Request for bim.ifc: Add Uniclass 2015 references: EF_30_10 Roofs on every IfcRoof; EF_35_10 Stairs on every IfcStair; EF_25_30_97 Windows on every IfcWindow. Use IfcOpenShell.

First a look at what the model holds.

```python
import ifcopenshell

model = ifcopenshell.open("bim.ifc")
print(model.schema)
print("classifications:", [c.Name for c in model.by_type("IfcClassification")])
for ifc_class in ("IfcDoor", "IfcRoof", "IfcStair", "IfcWall", "IfcWindow"):
    print(ifc_class, len(model.by_type(ifc_class)))
```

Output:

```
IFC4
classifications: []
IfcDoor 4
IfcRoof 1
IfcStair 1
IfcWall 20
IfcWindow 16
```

```python
import ifcopenshell
import ifcopenshell.api.classification

model = ifcopenshell.open("bim.ifc")

system = ifcopenshell.api.classification.add_classification(model, classification="Uniclass 2015")

codes = {
    "IfcRoof": ("EF_30_10", "Roofs"),
    "IfcStair": ("EF_35_10", "Stairs"),
    "IfcWindow": ("EF_25_30_97", "Windows"),
}
for ifc_class, (code, name) in codes.items():
    products = model.by_type(ifc_class)
    ifcopenshell.api.classification.add_reference(
        model, products=products, classification=system, identification=code, name=name
    )
    print(code, len(products))

model.write("bim_rev.ifc")
```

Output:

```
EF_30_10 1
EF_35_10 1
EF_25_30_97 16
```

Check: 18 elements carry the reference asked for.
